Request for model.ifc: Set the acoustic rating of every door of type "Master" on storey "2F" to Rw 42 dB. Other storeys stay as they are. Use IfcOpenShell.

First a look at what the model holds.

```python
import ifcopenshell
import ifcopenshell.util.element

model = ifcopenshell.open("model.ifc")
print(model.schema)
storey = next(s for s in model.by_type("IfcBuildingStorey") if s.Name == "2F")
doors = [e for e in ifcopenshell.util.element.get_decomposition(storey) if e.is_a("IfcDoor")]
seen = {}
for e in doors:
    element_type = ifcopenshell.util.element.get_type(e)
    key = (element_type.Name if element_type != e and element_type else None, ifcopenshell.util.element.get_pset(e, "Pset_DoorCommon", "AcousticRating"))
    seen[key] = seen.get(key, 0) + 1
for (name, value), count in sorted(seen.items(), key=str):
    print(count, "x", name, "|", value)
```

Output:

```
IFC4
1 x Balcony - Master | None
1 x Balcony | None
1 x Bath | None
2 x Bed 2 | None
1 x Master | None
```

```python
import ifcopenshell
import ifcopenshell.api.pset
import ifcopenshell.util.element

model = ifcopenshell.open("model.ifc")

storey = next(s for s in model.by_type("IfcBuildingStorey") if s.Name == "2F")
doors = [e for e in ifcopenshell.util.element.get_decomposition(storey) if e.is_a("IfcDoor")]

count = 0
for e in doors:
    element_type = ifcopenshell.util.element.get_type(e)
    if element_type in (None, e) or element_type.Name != "Master":
        continue
    # add_pset returns the element's existing set when there is one.
    pset = ifcopenshell.api.pset.add_pset(model, product=e, name="Pset_DoorCommon")
    ifcopenshell.api.pset.edit_pset(model, pset=pset, properties={"AcousticRating": "Rw 42 dB"})
    count += 1

print(count, "doors updated")

model.write("model_edited.ifc")
```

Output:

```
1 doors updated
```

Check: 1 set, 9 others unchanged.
